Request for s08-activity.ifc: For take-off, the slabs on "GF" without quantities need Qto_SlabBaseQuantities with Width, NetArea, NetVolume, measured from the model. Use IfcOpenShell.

First a look at what the model holds.

```python
import ifcopenshell
import ifcopenshell.util.element
import ifcopenshell.util.unit

model = ifcopenshell.open("s08-activity.ifc")
print(model.schema)
for unit_type in ("LENGTHUNIT", "AREAUNIT", "VOLUMEUNIT"):
    print(unit_type, ifcopenshell.util.unit.calculate_unit_scale(model, unit_type))
storey = next(s for s in model.by_type("IfcBuildingStorey") if s.Name == "GF")
slabs = [e for e in ifcopenshell.util.element.get_decomposition(storey) if e.is_a("IfcSlab")]
for e in sorted(slabs, key=lambda e: e.id()):
    print(e.id(), e.is_a(), e.Name, list(ifcopenshell.util.element.get_psets(e, qtos_only=True)), sep=" | ")
```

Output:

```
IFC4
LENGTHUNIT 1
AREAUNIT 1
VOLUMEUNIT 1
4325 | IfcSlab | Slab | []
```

```python
import ifcopenshell
import ifcopenshell.api.pset
import ifcopenshell.geom
import ifcopenshell.util.element
import ifcopenshell.util.shape
import ifcopenshell.util.unit

model = ifcopenshell.open("s08-activity.ifc")
unit_scale = ifcopenshell.util.unit.calculate_unit_scale(model)
area_scale = ifcopenshell.util.unit.calculate_unit_scale(model, "AREAUNIT")
volume_scale = ifcopenshell.util.unit.calculate_unit_scale(model, "VOLUMEUNIT")
settings = ifcopenshell.geom.settings()

storey = next(s for s in model.by_type("IfcBuildingStorey") if s.Name == "GF")
slabs = [e for e in ifcopenshell.util.element.get_decomposition(storey) if e.is_a("IfcSlab")]

for e in sorted(slabs, key=lambda e: e.id()):
    if ifcopenshell.util.element.get_psets(e, qtos_only=True, should_inherit=False):
        continue
    # Geometry comes back in metres, in the element's own axes.
    shape = ifcopenshell.geom.create_shape(settings, e)
    values = {
        "Width": ifcopenshell.util.shape.get_z(shape.geometry) / unit_scale,
        "NetArea": ifcopenshell.util.shape.get_footprint_area(shape.geometry) / area_scale,
        "NetVolume": ifcopenshell.util.shape.get_volume(shape.geometry) / volume_scale,
    }
    qto = ifcopenshell.api.pset.add_qto(model, product=e, name="Qto_SlabBaseQuantities")
    ifcopenshell.api.pset.edit_qto(model, qto=qto, properties=values)
    print(e.id(), {k: round(v, 3) for k, v in values.items()})

model.write("s08-activity-out.ifc")
```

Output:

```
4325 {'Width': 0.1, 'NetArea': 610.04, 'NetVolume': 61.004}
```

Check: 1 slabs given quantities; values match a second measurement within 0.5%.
